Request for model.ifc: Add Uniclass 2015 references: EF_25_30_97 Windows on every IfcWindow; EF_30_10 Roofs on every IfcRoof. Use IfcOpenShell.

First a look at what the model holds.

```python
import ifcopenshell

model = ifcopenshell.open("model.ifc")
print(model.schema)
print("classifications:", [c.Name for c in model.by_type("IfcClassification")])
for ifc_class in ("IfcDoor", "IfcRoof", "IfcStair", "IfcWall", "IfcWindow"):
    print(ifc_class, len(model.by_type(ifc_class)))
```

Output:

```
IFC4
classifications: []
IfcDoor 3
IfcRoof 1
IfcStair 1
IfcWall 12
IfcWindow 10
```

```python
import ifcopenshell
import ifcopenshell.api.classification

model = ifcopenshell.open("model.ifc")

system = ifcopenshell.api.classification.add_classification(model, classification="Uniclass 2015")

codes = {
    "IfcWindow": ("EF_25_30_97", "Windows"),
    "IfcRoof": ("EF_30_10", "Roofs"),
}
for ifc_class, (code, name) in codes.items():
    products = model.by_type(ifc_class)
    ifcopenshell.api.classification.add_reference(
        model, products=products, classification=system, identification=code, name=name
    )
    print(code, len(products))

model.write("model-out.ifc")
```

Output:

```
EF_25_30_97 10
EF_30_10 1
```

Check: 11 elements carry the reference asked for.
